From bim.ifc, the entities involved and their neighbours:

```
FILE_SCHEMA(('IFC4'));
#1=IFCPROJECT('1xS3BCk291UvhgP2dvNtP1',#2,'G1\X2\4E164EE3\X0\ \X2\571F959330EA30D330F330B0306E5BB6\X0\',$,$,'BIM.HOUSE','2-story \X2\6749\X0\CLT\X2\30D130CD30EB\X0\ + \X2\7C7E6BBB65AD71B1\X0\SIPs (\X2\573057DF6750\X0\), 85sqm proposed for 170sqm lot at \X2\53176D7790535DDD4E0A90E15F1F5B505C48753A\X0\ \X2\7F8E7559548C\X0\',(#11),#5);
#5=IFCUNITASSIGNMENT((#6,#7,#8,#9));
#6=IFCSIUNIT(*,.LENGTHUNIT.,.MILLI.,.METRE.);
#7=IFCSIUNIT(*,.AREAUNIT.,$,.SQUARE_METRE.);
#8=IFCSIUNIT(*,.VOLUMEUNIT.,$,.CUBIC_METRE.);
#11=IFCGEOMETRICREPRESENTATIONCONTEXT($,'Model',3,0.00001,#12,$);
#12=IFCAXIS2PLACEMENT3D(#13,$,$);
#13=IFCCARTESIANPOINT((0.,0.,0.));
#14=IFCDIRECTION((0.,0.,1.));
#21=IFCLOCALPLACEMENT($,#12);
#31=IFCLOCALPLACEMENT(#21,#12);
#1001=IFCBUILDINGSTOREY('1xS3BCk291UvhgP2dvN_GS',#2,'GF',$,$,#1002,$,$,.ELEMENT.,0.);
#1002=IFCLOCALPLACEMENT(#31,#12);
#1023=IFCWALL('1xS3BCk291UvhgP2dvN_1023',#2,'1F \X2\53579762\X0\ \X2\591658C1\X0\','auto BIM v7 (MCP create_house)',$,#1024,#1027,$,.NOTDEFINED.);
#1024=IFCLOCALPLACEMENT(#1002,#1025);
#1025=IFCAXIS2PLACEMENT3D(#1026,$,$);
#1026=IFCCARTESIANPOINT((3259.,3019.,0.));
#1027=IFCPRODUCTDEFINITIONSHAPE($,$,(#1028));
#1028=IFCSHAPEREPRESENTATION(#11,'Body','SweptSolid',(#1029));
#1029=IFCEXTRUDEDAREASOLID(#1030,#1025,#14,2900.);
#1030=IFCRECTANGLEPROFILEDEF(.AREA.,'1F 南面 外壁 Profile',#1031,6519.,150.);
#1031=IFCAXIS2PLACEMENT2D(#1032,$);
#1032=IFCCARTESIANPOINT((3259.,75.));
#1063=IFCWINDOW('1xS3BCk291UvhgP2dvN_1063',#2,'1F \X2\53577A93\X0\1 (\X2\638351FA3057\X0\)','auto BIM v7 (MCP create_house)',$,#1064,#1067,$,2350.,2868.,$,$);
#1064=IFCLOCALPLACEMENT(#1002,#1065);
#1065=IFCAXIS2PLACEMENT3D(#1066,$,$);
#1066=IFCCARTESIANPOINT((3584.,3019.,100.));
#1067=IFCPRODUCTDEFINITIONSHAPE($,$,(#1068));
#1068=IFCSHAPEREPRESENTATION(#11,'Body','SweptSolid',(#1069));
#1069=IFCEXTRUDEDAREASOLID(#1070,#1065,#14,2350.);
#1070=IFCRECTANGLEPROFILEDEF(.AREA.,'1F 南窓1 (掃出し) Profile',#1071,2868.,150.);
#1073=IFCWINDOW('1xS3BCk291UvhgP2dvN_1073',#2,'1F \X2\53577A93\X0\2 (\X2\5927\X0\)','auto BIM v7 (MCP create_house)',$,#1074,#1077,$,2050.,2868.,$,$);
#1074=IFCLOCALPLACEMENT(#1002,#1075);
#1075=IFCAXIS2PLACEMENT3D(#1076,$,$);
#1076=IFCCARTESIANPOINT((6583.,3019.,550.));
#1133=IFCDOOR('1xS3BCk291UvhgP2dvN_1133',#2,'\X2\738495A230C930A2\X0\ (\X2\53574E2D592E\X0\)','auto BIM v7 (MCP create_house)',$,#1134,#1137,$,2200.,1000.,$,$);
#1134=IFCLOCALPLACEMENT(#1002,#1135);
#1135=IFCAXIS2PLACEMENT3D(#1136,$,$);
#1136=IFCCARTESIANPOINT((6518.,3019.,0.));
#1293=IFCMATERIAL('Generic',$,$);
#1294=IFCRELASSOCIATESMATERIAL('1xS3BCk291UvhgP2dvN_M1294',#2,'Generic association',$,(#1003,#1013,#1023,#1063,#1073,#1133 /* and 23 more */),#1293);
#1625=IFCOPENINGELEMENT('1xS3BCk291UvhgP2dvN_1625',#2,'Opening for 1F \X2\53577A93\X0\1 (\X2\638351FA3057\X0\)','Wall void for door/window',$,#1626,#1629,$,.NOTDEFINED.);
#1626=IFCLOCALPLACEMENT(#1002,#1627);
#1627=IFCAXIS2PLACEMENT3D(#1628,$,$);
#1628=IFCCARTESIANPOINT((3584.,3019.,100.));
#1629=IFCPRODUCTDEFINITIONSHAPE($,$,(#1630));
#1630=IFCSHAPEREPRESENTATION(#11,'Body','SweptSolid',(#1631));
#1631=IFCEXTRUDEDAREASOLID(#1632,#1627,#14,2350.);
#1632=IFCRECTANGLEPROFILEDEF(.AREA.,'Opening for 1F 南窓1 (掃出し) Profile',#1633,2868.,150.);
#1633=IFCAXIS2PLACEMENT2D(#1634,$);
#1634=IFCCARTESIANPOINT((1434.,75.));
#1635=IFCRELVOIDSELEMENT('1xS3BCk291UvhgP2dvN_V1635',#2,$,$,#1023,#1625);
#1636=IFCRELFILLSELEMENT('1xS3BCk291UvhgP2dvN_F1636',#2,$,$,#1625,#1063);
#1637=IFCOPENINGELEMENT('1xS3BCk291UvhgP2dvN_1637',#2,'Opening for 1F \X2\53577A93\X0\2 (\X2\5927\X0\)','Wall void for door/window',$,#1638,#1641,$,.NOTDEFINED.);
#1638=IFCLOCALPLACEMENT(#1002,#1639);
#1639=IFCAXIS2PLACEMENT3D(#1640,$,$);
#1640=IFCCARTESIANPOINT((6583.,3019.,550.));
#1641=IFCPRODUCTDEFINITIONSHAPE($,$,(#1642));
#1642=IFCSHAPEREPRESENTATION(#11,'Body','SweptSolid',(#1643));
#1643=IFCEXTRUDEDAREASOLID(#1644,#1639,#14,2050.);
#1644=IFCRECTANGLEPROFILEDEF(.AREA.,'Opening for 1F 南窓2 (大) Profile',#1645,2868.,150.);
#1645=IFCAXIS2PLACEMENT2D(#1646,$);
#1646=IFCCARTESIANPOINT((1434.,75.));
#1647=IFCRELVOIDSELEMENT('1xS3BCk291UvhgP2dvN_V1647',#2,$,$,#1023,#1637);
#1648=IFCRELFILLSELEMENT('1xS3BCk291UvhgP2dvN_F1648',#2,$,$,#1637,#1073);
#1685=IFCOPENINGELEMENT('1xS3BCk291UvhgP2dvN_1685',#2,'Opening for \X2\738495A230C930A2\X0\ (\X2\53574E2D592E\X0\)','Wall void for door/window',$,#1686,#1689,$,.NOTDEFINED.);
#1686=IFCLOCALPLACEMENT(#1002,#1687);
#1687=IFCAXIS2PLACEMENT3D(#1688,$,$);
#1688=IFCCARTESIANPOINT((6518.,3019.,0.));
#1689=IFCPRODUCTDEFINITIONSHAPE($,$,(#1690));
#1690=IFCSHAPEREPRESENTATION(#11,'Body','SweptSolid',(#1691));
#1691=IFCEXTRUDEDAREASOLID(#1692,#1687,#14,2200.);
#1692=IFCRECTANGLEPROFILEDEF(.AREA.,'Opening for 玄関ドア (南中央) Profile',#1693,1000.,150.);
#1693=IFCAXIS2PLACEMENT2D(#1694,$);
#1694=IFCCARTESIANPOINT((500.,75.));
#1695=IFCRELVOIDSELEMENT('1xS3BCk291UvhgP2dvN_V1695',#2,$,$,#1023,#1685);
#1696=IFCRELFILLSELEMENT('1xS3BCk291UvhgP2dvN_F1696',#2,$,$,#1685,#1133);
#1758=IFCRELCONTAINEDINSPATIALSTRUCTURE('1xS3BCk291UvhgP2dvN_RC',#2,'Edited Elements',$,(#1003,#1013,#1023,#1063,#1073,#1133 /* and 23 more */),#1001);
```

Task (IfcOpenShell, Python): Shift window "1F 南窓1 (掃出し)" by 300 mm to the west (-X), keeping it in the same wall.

```python
import ifcopenshell
import ifcopenshell.api.geometry
import ifcopenshell.util.placement
import ifcopenshell.util.unit

model = ifcopenshell.open("bim.ifc")
unit_scale = ifcopenshell.util.unit.calculate_unit_scale(model)

window = model.by_guid("1xS3BCk291UvhgP2dvN_1063")
opening = window.FillsVoids[0].RelatingOpeningElement
wall = opening.VoidsElements[0].RelatingBuildingElement

wall_matrix = ifcopenshell.util.placement.get_local_placement(wall.ObjectPlacement)
shift = wall_matrix[:3, 0] * -0.3 / unit_scale
before = ifcopenshell.util.placement.get_local_placement(window.ObjectPlacement)[:3, 3].copy()

# The window is not placed relative to its opening, so move both.
for product in (opening, window):
    matrix = ifcopenshell.util.placement.get_local_placement(product.ObjectPlacement)
    matrix[:3, 3] += shift
    ifcopenshell.api.geometry.edit_object_placement(model, product=product, matrix=matrix, is_si=False)

after = ifcopenshell.util.placement.get_local_placement(window.ObjectPlacement)[:3, 3]
print("window moved by", (after - before).round(3) + 0.0)

model.write("bim_edited.ifc")
```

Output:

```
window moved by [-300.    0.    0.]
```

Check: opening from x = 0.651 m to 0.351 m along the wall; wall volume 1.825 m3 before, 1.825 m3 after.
